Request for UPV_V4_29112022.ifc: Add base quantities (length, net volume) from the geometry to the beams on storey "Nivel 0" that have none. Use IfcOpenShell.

First a look at what the model holds.

```python
import ifcopenshell
import ifcopenshell.util.element
import ifcopenshell.util.unit

model = ifcopenshell.open("UPV_V4_29112022.ifc")
print(model.schema)
for unit_type in ("LENGTHUNIT", "AREAUNIT", "VOLUMEUNIT"):
    print(unit_type, ifcopenshell.util.unit.calculate_unit_scale(model, unit_type))
storey = next(s for s in model.by_type("IfcBuildingStorey") if s.Name == "Nivel 0")
beams = [e for e in ifcopenshell.util.element.get_decomposition(storey) if e.is_a("IfcBeam")]
for e in sorted(beams, key=lambda e: e.id()):
    print(e.id(), e.is_a(), e.Name, list(ifcopenshell.util.element.get_psets(e, qtos_only=True)), sep=" | ")
```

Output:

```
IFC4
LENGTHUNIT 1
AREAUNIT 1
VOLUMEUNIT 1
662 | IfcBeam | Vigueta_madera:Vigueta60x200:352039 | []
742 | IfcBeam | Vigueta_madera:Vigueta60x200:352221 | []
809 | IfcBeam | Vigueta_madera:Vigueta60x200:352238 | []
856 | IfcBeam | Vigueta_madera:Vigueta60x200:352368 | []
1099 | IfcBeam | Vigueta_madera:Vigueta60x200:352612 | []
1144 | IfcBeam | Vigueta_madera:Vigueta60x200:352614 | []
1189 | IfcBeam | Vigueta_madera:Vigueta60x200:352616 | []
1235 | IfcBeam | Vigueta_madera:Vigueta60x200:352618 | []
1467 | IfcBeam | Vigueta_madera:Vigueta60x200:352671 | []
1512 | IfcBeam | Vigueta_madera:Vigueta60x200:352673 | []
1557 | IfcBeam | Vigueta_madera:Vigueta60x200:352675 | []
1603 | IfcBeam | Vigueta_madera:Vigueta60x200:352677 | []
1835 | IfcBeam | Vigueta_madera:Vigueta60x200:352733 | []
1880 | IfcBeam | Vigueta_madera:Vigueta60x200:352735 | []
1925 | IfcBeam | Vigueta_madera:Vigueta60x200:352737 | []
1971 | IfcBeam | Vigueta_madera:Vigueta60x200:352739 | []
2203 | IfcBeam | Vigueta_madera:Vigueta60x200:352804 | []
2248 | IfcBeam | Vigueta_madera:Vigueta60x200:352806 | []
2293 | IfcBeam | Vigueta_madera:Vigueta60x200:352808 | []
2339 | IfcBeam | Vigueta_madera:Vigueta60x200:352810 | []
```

```python
import ifcopenshell
import ifcopenshell.api.pset
import ifcopenshell.geom
import ifcopenshell.util.element
import ifcopenshell.util.shape
import ifcopenshell.util.unit

model = ifcopenshell.open("UPV_V4_29112022.ifc")
unit_scale = ifcopenshell.util.unit.calculate_unit_scale(model)
volume_scale = ifcopenshell.util.unit.calculate_unit_scale(model, "VOLUMEUNIT")
settings = ifcopenshell.geom.settings()

storey = next(s for s in model.by_type("IfcBuildingStorey") if s.Name == "Nivel 0")
beams = [e for e in ifcopenshell.util.element.get_decomposition(storey) if e.is_a("IfcBeam")]

for e in sorted(beams, key=lambda e: e.id()):
    if ifcopenshell.util.element.get_psets(e, qtos_only=True, should_inherit=False):
        continue
    # Geometry comes back in metres, in the element's own axes.
    shape = ifcopenshell.geom.create_shape(settings, e)
    values = {
        "Length": ifcopenshell.util.shape.get_max_xyz(shape.geometry) / unit_scale,
        "NetVolume": ifcopenshell.util.shape.get_volume(shape.geometry) / volume_scale,
    }
    qto = ifcopenshell.api.pset.add_qto(model, product=e, name="Qto_BeamBaseQuantities")
    ifcopenshell.api.pset.edit_qto(model, qto=qto, properties=values)
    print(e.id(), {k: round(v, 3) for k, v in values.items()})

model.write("UPV_V4_29112022_rev.ifc")
```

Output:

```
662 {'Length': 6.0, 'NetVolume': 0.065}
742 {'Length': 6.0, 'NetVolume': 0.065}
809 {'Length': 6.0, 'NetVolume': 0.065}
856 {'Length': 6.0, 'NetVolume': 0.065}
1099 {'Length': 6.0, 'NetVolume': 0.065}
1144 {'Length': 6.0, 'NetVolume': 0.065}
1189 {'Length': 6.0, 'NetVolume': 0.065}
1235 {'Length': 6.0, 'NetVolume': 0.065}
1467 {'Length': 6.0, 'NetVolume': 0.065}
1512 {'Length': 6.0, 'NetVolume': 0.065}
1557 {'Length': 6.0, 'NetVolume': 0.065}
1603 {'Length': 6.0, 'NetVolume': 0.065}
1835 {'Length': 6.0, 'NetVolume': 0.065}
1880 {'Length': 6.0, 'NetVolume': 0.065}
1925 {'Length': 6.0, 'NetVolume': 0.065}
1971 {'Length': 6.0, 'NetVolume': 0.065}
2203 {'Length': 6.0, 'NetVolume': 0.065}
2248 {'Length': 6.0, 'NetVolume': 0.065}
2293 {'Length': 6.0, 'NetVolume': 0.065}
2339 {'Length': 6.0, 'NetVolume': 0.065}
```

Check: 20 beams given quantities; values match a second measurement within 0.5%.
